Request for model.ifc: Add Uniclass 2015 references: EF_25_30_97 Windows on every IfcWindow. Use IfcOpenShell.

First a look at what the model holds.

```python
import ifcopenshell

model = ifcopenshell.open("model.ifc")
print(model.schema)
print("classifications:", [c.Name for c in model.by_type("IfcClassification")])
for ifc_class in ("IfcDoor", "IfcRoof", "IfcStair", "IfcWall", "IfcWindow"):
    print(ifc_class, len(model.by_type(ifc_class)))
```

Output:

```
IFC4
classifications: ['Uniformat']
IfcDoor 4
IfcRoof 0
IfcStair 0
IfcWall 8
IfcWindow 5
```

```python
import ifcopenshell
import ifcopenshell.api.classification

model = ifcopenshell.open("model.ifc")

system = ifcopenshell.api.classification.add_classification(model, classification="Uniclass 2015")

codes = {
    "IfcWindow": ("EF_25_30_97", "Windows"),
}
for ifc_class, (code, name) in codes.items():
    products = model.by_type(ifc_class)
    ifcopenshell.api.classification.add_reference(
        model, products=products, classification=system, identification=code, name=name
    )
    print(code, len(products))

model.write("model-out.ifc")
```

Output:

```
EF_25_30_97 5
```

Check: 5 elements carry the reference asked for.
